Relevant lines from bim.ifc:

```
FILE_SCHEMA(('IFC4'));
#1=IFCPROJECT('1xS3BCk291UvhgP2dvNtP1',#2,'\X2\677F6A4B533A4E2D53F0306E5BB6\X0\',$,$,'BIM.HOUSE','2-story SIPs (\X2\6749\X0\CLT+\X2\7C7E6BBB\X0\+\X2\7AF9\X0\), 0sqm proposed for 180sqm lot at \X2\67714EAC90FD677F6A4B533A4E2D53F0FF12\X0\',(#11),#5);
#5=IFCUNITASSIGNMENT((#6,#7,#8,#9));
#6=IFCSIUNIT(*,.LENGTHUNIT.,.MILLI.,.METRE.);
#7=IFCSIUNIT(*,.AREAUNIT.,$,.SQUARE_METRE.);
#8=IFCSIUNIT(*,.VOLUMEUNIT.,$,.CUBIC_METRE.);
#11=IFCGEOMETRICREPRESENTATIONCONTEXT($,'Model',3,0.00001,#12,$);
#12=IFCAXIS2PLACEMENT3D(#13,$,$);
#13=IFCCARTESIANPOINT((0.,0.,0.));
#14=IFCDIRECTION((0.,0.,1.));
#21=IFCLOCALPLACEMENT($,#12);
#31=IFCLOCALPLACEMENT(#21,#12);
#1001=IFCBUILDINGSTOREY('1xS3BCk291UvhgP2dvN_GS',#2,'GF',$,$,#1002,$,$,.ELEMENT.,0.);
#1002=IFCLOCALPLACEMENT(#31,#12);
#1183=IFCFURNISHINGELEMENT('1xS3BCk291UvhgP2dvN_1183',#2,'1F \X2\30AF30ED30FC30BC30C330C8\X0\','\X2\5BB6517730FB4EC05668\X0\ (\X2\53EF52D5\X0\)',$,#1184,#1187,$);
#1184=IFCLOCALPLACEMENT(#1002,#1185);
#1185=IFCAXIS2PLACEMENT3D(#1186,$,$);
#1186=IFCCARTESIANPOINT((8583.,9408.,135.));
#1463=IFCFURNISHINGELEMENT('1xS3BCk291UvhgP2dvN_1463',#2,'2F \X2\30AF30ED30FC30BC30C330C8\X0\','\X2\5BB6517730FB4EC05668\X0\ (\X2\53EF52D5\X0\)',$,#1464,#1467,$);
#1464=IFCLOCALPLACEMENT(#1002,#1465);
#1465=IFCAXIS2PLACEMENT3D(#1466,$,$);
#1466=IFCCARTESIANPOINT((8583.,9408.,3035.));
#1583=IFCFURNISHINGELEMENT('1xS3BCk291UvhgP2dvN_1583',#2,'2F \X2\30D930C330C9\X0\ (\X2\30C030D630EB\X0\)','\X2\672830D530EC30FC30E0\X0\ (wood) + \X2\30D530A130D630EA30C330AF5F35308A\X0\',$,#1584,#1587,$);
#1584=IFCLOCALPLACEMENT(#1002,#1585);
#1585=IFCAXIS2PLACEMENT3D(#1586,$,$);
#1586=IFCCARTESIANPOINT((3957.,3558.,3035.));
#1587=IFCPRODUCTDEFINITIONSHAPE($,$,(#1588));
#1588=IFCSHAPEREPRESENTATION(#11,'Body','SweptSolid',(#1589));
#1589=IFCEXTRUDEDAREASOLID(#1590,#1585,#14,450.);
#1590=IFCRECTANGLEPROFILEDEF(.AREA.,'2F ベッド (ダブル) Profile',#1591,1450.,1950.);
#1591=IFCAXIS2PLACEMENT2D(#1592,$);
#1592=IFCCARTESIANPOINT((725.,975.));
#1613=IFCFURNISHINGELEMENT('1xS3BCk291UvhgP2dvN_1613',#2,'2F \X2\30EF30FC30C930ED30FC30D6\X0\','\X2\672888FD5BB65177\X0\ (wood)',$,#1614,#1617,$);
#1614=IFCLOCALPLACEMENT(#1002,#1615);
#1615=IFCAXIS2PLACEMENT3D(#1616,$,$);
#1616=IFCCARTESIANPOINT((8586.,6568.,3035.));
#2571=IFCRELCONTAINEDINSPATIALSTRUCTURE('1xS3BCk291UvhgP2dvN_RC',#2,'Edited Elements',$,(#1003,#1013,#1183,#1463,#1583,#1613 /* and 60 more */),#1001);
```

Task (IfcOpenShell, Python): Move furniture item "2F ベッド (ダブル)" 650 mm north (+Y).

```python
import ifcopenshell
import ifcopenshell.api.geometry
import ifcopenshell.util.placement
import ifcopenshell.util.unit

model = ifcopenshell.open("bim.ifc")
unit_scale = ifcopenshell.util.unit.calculate_unit_scale(model)

item = model.by_guid("1xS3BCk291UvhgP2dvN_1583")
matrix = ifcopenshell.util.placement.get_local_placement(item.ObjectPlacement)
matrix[1, 3] += 0.65 / unit_scale
ifcopenshell.api.geometry.edit_object_placement(model, product=item, matrix=matrix, is_si=False)

print(ifcopenshell.util.placement.get_local_placement(item.ObjectPlacement).round(3) + 0.0)

model.write("bim_edited.ifc")
```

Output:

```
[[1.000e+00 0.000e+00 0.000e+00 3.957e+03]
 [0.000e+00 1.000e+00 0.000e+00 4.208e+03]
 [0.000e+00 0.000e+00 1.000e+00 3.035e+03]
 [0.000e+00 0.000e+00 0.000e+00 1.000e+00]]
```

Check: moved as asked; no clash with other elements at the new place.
